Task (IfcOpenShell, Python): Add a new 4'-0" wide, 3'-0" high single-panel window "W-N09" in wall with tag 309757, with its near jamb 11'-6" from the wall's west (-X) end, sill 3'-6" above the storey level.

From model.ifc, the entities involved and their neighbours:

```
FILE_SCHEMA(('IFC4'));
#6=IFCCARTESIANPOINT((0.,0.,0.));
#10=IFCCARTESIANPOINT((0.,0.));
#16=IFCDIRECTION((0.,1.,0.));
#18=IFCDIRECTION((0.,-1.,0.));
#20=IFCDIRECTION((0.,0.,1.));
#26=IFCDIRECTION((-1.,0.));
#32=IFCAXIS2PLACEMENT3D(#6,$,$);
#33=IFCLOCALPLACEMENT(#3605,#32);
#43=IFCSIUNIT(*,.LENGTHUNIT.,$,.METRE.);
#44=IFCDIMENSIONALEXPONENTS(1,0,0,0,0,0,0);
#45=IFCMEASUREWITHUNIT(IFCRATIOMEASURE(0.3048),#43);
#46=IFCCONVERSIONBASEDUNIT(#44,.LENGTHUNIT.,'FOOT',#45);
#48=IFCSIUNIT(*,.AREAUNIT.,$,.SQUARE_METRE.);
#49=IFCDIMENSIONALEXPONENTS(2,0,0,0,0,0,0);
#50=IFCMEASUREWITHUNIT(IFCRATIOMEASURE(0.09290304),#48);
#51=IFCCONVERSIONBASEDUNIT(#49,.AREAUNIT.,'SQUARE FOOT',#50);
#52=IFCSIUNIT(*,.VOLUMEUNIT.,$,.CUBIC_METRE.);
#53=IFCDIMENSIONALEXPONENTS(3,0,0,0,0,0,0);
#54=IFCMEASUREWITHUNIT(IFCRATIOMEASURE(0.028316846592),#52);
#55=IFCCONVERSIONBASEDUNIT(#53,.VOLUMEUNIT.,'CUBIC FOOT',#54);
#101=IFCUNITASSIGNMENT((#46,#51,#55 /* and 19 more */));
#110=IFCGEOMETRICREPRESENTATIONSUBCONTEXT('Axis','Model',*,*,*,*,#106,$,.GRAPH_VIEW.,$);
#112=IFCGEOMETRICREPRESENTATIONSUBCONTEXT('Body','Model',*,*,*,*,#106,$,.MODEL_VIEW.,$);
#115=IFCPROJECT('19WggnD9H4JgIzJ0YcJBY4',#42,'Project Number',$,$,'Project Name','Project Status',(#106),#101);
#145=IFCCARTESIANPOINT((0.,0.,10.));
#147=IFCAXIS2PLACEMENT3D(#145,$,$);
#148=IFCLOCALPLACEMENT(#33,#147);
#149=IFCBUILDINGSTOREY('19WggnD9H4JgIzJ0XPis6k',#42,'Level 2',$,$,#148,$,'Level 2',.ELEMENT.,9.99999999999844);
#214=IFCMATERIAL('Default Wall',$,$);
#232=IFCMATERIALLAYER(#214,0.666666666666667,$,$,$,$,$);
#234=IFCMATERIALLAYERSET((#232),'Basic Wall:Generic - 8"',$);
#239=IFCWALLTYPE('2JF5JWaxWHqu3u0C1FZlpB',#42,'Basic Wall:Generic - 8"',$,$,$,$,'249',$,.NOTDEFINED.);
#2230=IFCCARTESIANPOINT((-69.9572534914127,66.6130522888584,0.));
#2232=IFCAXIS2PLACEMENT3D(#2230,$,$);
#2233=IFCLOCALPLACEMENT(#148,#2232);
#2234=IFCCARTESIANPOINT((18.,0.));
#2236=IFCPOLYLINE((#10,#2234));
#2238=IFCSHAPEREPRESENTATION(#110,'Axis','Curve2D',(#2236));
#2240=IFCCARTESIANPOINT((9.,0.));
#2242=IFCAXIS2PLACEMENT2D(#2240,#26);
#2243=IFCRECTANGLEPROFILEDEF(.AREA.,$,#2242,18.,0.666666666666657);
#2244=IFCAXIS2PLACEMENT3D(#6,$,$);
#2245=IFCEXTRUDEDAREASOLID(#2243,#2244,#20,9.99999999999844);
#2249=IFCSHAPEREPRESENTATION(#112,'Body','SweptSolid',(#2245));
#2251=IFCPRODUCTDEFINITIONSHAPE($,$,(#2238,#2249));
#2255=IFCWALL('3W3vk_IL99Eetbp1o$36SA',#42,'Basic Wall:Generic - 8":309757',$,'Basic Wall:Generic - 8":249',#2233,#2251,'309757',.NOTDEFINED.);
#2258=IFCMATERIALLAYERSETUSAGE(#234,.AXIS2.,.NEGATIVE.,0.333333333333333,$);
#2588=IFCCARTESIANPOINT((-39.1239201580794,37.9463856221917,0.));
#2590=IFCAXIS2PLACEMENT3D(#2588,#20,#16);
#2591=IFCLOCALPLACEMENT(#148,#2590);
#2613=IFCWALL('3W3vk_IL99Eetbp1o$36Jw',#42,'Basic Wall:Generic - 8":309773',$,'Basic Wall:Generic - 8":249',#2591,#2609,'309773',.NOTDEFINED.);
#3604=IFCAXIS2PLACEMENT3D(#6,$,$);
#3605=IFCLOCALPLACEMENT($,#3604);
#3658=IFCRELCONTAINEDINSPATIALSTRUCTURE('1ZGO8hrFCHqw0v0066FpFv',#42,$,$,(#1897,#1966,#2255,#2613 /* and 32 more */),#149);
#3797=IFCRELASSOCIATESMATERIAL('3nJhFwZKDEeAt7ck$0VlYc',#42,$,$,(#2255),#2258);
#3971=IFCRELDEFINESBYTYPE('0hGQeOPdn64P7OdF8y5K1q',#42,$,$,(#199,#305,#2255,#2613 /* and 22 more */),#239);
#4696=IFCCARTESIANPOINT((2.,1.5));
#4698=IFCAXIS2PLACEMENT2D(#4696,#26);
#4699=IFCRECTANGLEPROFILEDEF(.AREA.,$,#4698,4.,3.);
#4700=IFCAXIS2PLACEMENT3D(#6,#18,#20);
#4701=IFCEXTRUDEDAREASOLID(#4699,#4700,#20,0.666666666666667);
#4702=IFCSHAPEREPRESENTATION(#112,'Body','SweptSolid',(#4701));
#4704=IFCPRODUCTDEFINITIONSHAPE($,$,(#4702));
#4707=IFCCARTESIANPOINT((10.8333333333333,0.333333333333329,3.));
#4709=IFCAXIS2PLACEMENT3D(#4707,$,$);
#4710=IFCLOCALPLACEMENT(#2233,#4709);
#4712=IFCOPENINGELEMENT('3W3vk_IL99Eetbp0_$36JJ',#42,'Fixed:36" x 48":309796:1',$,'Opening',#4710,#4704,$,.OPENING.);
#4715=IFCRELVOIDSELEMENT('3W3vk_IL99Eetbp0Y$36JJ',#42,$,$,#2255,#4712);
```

```python
import numpy as np
import ifcopenshell
import ifcopenshell.api.feature
import ifcopenshell.api.geometry
import ifcopenshell.api.root
import ifcopenshell.api.spatial
import ifcopenshell.geom
import ifcopenshell.util.element
import ifcopenshell.util.placement
import ifcopenshell.util.representation
import ifcopenshell.util.shape
import ifcopenshell.util.unit

model = ifcopenshell.open("model.ifc")
unit_scale = ifcopenshell.util.unit.calculate_unit_scale(model)
settings = ifcopenshell.geom.settings()


def volume(element):
    """Net volume in cubic metres, openings subtracted."""
    shape = ifcopenshell.geom.create_shape(settings, element)
    return ifcopenshell.util.shape.get_volume(shape.geometry)


wall = model.by_guid("3W3vk_IL99Eetbp1o$36SA")
storey = ifcopenshell.util.element.get_container(wall, ifc_class="IfcBuildingStorey")
context = ifcopenshell.util.representation.get_context(model, "Model", "Body", "MODEL_VIEW")
before = volume(wall)

width, height, from_end, sill = 1.2192, 0.9144, 3.5052, 1.0668  # metres

# The wall runs along its own X axis, and the end named is its -X end.
wall_shape = ifcopenshell.geom.create_shape(settings, wall)
x, y, z = ifcopenshell.util.shape.get_vertices(wall_shape.geometry).T
start = x.min() + from_end
face, thickness = float(y.min()), float(y.max() - y.min())
wall_matrix = ifcopenshell.util.placement.get_local_placement(wall.ObjectPlacement)
level = ifcopenshell.util.placement.get_local_placement(storey.ObjectPlacement)[2, 3]


def in_wall(x, y):
    """Placement at x, y metres in the wall's axes, at sill height."""
    matrix = wall_matrix.copy()
    matrix[:, 3] = wall_matrix @ np.array([x / unit_scale, y / unit_scale, 0.0, 1.0])
    matrix[2, 3] = level + sill / unit_scale
    return matrix


# Opening: a box that overshoots both wall faces by 50 mm.
opening = ifcopenshell.api.root.create_entity(model, ifc_class="IfcOpeningElement", predefined_type="OPENING")
box = ifcopenshell.api.geometry.add_wall_representation(
    model, context=context, length=width, height=height, thickness=thickness + 0.1
)
ifcopenshell.api.geometry.assign_representation(model, product=opening, representation=box)
ifcopenshell.api.geometry.edit_object_placement(model, product=opening, matrix=in_wall(start, face - 0.05), is_si=False)
ifcopenshell.api.feature.add_feature(model, feature=opening, element=wall)

window = ifcopenshell.api.root.create_entity(model, ifc_class="IfcWindow", name="W-N09", predefined_type="WINDOW")
window.OverallWidth, window.OverallHeight = width / unit_scale, height / unit_scale
window.PartitioningType = "SINGLE_PANEL"
body = ifcopenshell.api.geometry.add_window_representation(
    model,
    context=context,
    overall_width=window.OverallWidth,
    overall_height=window.OverallHeight,
    partition_type="SINGLE_PANEL",
)
ifcopenshell.api.geometry.assign_representation(model, product=window, representation=body)
ifcopenshell.api.spatial.assign_container(model, products=[window], relating_structure=storey)
ifcopenshell.api.feature.add_filling(model, opening=opening, element=window)

# Centre the window in the wall's thickness.
ifcopenshell.api.geometry.edit_object_placement(model, product=window, matrix=in_wall(start, face), is_si=False)
window_shape = ifcopenshell.geom.create_shape(settings, window)
depth = ifcopenshell.util.shape.get_vertices(window_shape.geometry)[:, 1]
offset = face + thickness / 2 - (depth.min() + depth.max()) / 2
ifcopenshell.api.geometry.edit_object_placement(model, product=window, matrix=in_wall(start, offset), is_si=False)

after = volume(wall)

print(f"wall volume {before:.3f} -> {after:.3f} m3")

model.write("model_edited.ifc")
```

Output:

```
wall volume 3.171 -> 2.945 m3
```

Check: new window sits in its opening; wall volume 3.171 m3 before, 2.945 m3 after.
